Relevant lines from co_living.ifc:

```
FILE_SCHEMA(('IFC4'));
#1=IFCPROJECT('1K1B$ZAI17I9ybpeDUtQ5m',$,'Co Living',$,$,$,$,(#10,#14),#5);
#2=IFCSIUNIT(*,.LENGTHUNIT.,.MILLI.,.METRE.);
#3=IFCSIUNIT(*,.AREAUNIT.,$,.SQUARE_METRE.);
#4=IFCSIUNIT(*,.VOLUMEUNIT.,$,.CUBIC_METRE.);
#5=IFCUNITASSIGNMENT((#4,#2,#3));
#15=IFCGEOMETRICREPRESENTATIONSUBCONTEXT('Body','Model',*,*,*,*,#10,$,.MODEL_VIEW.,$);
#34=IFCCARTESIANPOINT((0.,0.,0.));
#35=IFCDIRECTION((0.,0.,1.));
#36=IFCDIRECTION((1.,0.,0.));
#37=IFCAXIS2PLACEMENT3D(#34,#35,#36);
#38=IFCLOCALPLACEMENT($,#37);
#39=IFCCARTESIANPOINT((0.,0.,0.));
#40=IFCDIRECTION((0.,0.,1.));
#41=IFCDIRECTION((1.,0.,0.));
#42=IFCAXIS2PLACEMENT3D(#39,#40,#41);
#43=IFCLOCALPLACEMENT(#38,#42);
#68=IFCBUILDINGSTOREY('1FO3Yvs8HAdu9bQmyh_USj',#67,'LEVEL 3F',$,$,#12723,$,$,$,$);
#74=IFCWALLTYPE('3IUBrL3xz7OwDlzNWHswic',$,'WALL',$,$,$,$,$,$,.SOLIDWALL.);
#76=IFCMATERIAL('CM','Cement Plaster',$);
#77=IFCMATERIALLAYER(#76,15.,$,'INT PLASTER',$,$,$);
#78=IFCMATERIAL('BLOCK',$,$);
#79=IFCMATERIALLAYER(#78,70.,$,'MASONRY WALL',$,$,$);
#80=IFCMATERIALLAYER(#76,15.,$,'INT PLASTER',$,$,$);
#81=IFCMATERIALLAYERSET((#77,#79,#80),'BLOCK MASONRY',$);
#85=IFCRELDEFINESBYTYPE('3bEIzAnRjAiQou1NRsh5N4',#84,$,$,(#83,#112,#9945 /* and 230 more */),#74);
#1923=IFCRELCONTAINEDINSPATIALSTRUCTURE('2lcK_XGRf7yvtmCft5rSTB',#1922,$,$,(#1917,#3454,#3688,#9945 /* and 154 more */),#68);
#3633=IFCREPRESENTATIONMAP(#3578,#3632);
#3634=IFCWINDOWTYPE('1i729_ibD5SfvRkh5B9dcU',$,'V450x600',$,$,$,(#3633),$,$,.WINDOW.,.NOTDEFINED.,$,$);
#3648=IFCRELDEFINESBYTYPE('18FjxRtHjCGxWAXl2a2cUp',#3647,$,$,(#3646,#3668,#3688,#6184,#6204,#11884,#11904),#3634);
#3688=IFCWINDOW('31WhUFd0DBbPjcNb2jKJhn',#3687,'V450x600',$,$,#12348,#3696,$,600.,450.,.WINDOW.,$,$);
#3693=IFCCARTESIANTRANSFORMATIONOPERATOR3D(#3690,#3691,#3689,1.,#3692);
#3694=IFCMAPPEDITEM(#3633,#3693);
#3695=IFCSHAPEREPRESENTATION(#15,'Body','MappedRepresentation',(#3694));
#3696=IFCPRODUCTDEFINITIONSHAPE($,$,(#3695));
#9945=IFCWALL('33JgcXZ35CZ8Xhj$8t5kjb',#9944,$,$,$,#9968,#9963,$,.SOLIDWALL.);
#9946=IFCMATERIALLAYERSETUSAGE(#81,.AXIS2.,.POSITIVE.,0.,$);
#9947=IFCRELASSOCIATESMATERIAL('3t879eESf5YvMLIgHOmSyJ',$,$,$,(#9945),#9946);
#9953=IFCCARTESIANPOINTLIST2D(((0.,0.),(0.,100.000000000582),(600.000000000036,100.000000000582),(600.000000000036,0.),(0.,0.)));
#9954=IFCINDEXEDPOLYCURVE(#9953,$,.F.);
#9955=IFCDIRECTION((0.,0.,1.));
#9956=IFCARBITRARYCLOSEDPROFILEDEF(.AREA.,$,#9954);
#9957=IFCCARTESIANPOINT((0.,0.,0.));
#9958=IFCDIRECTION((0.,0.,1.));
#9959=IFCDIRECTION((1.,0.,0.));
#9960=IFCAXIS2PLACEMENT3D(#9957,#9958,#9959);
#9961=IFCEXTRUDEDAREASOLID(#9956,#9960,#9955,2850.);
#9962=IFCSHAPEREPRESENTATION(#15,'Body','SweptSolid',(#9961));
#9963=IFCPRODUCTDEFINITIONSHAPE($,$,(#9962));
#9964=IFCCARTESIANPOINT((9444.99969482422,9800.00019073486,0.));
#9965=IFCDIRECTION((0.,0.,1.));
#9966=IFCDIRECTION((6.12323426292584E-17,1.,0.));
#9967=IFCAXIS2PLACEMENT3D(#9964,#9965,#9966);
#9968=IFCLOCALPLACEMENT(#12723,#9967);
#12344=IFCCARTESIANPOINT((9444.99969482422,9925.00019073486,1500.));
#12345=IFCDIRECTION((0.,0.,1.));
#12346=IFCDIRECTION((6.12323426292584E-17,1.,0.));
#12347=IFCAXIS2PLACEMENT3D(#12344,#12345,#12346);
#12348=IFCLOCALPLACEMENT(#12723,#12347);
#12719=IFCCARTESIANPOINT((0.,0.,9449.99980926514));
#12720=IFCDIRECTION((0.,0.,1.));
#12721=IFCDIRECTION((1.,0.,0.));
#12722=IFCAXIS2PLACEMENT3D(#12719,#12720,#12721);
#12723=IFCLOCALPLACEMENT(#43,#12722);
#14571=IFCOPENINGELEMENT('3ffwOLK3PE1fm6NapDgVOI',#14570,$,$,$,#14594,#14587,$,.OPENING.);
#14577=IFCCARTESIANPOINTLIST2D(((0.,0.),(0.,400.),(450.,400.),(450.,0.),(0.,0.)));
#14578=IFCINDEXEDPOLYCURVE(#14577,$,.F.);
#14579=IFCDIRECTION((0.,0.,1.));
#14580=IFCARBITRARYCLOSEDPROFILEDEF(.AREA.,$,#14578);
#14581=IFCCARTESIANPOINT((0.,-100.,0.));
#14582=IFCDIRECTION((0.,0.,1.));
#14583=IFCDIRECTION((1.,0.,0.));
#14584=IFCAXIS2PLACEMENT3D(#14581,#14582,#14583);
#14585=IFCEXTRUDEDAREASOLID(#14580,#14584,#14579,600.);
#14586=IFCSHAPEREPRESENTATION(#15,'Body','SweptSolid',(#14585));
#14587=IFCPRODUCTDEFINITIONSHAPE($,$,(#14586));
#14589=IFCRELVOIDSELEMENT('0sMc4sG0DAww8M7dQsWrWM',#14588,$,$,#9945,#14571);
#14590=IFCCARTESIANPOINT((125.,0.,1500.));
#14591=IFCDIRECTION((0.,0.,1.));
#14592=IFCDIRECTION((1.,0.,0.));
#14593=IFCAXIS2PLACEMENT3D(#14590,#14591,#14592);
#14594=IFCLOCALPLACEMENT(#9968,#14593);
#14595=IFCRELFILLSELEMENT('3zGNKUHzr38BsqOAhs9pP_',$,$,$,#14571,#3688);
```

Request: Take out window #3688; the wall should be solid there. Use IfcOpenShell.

```python
import ifcopenshell
import ifcopenshell.api.feature
import ifcopenshell.api.root
import ifcopenshell.geom
import ifcopenshell.util.shape

model = ifcopenshell.open("co_living.ifc")
settings = ifcopenshell.geom.settings()


def volume(element):
    """Net volume in cubic metres, openings subtracted."""
    shape = ifcopenshell.geom.create_shape(settings, element)
    return ifcopenshell.util.shape.get_volume(shape.geometry)


window = model.by_guid("31WhUFd0DBbPjcNb2jKJhn")
opening = window.FillsVoids[0].RelatingOpeningElement
wall = opening.VoidsElements[0].RelatingBuildingElement
before = volume(wall)

ifcopenshell.api.root.remove_product(model, product=window)
ifcopenshell.api.feature.remove_feature(model, feature=opening)

after = volume(wall)

print(f"wall volume {before:.3f} -> {after:.3f} m3")

model.write("co_living_rev.ifc")
```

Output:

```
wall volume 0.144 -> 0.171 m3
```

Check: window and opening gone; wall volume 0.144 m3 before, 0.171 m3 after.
